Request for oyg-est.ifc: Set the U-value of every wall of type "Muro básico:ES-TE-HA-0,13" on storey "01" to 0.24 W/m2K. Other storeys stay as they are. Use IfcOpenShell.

First a look at what the model holds.

```python
import ifcopenshell
import ifcopenshell.util.element

model = ifcopenshell.open("oyg-est.ifc")
print(model.schema)
storey = next(s for s in model.by_type("IfcBuildingStorey") if s.Name == "01")
walls = [e for e in ifcopenshell.util.element.get_decomposition(storey) if e.is_a("IfcWall")]
seen = {}
for e in walls:
    element_type = ifcopenshell.util.element.get_type(e)
    key = (element_type.Name if element_type != e and element_type else None, ifcopenshell.util.element.get_pset(e, "Pset_WallCommon", "ThermalTransmittance"))
    seen[key] = seen.get(key, 0) + 1
for (name, value), count in sorted(seen.items(), key=str):
    print(count, "x", name, "|", value)
```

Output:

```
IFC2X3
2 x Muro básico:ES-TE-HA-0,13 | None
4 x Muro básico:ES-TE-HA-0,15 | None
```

```python
import ifcopenshell
import ifcopenshell.api.pset
import ifcopenshell.util.element

model = ifcopenshell.open("oyg-est.ifc")

storey = next(s for s in model.by_type("IfcBuildingStorey") if s.Name == "01")
walls = [e for e in ifcopenshell.util.element.get_decomposition(storey) if e.is_a("IfcWall")]

count = 0
for e in walls:
    element_type = ifcopenshell.util.element.get_type(e)
    if element_type in (None, e) or element_type.Name != "Muro básico:ES-TE-HA-0,13":
        continue
    # add_pset returns the element's existing set when there is one.
    pset = ifcopenshell.api.pset.add_pset(model, product=e, name="Pset_WallCommon")
    ifcopenshell.api.pset.edit_pset(model, pset=pset, properties={"ThermalTransmittance": 0.24})
    count += 1

print(count, "walls updated")

model.write("oyg-est_edited.ifc")
```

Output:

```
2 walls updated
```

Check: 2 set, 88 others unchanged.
